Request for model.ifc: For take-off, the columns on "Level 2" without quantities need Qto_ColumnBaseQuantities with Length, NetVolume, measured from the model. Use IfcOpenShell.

First a look at what the model holds.

```python
import ifcopenshell
import ifcopenshell.util.element
import ifcopenshell.util.unit

model = ifcopenshell.open("model.ifc")
print(model.schema)
for unit_type in ("LENGTHUNIT", "AREAUNIT", "VOLUMEUNIT"):
    print(unit_type, ifcopenshell.util.unit.calculate_unit_scale(model, unit_type))
storey = next(s for s in model.by_type("IfcBuildingStorey") if s.Name == "Level 2")
columns = [e for e in ifcopenshell.util.element.get_decomposition(storey) if e.is_a("IfcColumn")]
for e in sorted(columns, key=lambda e: e.id()):
    print(e.id(), e.is_a(), e.Name, list(ifcopenshell.util.element.get_psets(e, qtos_only=True)), sep=" | ")
```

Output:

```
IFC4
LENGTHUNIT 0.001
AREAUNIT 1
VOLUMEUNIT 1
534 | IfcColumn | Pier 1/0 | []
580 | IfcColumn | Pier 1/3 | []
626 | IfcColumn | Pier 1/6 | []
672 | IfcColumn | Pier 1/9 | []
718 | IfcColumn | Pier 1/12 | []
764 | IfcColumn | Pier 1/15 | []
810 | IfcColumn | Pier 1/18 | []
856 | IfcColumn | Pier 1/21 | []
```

```python
import ifcopenshell
import ifcopenshell.api.pset
import ifcopenshell.geom
import ifcopenshell.util.element
import ifcopenshell.util.shape
import ifcopenshell.util.unit

model = ifcopenshell.open("model.ifc")
unit_scale = ifcopenshell.util.unit.calculate_unit_scale(model)
volume_scale = ifcopenshell.util.unit.calculate_unit_scale(model, "VOLUMEUNIT")
settings = ifcopenshell.geom.settings()

storey = next(s for s in model.by_type("IfcBuildingStorey") if s.Name == "Level 2")
columns = [e for e in ifcopenshell.util.element.get_decomposition(storey) if e.is_a("IfcColumn")]

for e in sorted(columns, key=lambda e: e.id()):
    if ifcopenshell.util.element.get_psets(e, qtos_only=True, should_inherit=False):
        continue
    # Geometry comes back in metres, in the element's own axes.
    shape = ifcopenshell.geom.create_shape(settings, e)
    values = {
        "Length": ifcopenshell.util.shape.get_z(shape.geometry) / unit_scale,
        "NetVolume": ifcopenshell.util.shape.get_volume(shape.geometry) / volume_scale,
    }
    qto = ifcopenshell.api.pset.add_qto(model, product=e, name="Qto_ColumnBaseQuantities")
    ifcopenshell.api.pset.edit_qto(model, qto=qto, properties=values)
    print(e.id(), {k: round(v, 3) for k, v in values.items()})

model.write("model_edited.ifc")
```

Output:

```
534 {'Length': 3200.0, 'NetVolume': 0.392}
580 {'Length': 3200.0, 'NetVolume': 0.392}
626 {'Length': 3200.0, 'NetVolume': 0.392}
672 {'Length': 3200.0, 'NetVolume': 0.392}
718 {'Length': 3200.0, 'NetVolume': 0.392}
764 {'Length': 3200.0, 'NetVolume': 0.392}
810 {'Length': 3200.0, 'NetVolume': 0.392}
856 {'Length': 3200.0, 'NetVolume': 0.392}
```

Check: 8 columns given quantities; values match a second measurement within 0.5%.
